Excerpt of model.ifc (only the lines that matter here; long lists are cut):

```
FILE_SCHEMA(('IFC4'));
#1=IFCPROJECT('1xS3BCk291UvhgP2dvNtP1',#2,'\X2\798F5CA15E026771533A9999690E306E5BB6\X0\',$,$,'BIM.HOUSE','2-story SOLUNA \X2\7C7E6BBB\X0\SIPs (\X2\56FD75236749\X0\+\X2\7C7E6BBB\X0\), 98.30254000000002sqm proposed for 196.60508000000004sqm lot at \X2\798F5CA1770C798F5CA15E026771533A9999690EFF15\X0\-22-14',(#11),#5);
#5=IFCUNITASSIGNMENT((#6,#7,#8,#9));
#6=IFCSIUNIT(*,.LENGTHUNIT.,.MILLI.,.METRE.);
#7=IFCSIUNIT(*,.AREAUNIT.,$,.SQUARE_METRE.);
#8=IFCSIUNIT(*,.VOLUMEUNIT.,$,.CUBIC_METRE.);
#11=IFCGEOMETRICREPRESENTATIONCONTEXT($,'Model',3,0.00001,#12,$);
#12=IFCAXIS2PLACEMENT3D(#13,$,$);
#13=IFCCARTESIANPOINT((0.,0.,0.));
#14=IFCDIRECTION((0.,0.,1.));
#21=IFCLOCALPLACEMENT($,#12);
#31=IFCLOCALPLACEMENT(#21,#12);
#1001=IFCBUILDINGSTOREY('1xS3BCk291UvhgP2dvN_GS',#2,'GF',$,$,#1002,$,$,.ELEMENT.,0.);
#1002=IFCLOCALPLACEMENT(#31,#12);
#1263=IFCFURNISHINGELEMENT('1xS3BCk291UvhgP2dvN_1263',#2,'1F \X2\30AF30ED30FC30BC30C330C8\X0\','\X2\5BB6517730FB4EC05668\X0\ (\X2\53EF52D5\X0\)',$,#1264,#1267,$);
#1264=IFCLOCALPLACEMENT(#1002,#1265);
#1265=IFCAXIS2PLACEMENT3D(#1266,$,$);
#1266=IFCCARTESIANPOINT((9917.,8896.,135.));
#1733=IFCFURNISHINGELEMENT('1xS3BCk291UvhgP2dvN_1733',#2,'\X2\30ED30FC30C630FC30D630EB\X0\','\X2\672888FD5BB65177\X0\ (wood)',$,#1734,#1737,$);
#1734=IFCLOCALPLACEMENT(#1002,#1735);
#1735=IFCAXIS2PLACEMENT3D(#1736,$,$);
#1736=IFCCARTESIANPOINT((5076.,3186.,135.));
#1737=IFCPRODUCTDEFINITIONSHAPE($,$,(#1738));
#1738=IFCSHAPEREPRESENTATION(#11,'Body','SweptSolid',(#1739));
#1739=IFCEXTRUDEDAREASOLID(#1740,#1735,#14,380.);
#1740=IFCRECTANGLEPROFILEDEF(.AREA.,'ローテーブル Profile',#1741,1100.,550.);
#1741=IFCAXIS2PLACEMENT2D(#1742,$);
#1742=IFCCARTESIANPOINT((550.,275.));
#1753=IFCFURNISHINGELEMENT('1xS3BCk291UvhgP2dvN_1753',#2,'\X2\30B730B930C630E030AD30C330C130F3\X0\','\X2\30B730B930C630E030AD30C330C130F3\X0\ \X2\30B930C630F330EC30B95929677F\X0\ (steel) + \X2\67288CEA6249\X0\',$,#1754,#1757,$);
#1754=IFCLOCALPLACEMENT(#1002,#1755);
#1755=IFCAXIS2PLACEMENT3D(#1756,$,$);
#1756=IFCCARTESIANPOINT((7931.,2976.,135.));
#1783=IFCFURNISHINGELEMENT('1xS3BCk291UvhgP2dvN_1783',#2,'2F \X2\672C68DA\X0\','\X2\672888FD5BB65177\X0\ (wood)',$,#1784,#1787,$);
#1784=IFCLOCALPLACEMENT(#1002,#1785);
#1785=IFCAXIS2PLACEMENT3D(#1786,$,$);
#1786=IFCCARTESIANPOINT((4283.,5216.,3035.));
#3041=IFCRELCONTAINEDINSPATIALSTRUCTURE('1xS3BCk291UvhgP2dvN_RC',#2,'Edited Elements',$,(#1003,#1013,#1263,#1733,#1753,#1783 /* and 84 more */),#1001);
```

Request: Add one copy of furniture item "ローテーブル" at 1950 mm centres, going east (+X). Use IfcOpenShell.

```python
import numpy as np
import ifcopenshell
import ifcopenshell.api.geometry
import ifcopenshell.api.root
import ifcopenshell.util.element
import ifcopenshell.util.placement
import ifcopenshell.util.unit

model = ifcopenshell.open("model.ifc")
unit_scale = ifcopenshell.util.unit.calculate_unit_scale(model)


def reuse_history(source, copy):
    """copy_class also copies each property set's owner history, people and application; keep the originals."""
    for rel in copy.IsDefinedBy:
        if rel.is_a("IfcRelDefinesByProperties") and (history := rel.RelatingPropertyDefinition.OwnerHistory):
            rel.RelatingPropertyDefinition.OwnerHistory = source.OwnerHistory
            ifcopenshell.util.element.remove_deep2(model, history)


source = model.by_guid("1xS3BCk291UvhgP2dvN_1733")
base = ifcopenshell.util.placement.get_local_placement(source.ObjectPlacement)
step = np.array([1.0, 0.0, 0.0]) * 1.95 / unit_scale

for i in range(1, 2):
    copy = ifcopenshell.api.root.copy_class(model, product=source)
    copy.Representation = ifcopenshell.util.element.copy_deep(
        model, source.Representation, exclude=["IfcGeometricRepresentationContext", "IfcRepresentationMap"]
    )
    reuse_history(source, copy)
    matrix = base.copy()
    matrix[:3, 3] += i * step
    print("added at", matrix[:3, 3].round(3) + 0.0)
    ifcopenshell.api.geometry.edit_object_placement(model, product=copy, matrix=matrix, is_si=False)

model.write("model-out.ifc")
```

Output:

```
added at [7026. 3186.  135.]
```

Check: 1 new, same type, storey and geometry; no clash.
